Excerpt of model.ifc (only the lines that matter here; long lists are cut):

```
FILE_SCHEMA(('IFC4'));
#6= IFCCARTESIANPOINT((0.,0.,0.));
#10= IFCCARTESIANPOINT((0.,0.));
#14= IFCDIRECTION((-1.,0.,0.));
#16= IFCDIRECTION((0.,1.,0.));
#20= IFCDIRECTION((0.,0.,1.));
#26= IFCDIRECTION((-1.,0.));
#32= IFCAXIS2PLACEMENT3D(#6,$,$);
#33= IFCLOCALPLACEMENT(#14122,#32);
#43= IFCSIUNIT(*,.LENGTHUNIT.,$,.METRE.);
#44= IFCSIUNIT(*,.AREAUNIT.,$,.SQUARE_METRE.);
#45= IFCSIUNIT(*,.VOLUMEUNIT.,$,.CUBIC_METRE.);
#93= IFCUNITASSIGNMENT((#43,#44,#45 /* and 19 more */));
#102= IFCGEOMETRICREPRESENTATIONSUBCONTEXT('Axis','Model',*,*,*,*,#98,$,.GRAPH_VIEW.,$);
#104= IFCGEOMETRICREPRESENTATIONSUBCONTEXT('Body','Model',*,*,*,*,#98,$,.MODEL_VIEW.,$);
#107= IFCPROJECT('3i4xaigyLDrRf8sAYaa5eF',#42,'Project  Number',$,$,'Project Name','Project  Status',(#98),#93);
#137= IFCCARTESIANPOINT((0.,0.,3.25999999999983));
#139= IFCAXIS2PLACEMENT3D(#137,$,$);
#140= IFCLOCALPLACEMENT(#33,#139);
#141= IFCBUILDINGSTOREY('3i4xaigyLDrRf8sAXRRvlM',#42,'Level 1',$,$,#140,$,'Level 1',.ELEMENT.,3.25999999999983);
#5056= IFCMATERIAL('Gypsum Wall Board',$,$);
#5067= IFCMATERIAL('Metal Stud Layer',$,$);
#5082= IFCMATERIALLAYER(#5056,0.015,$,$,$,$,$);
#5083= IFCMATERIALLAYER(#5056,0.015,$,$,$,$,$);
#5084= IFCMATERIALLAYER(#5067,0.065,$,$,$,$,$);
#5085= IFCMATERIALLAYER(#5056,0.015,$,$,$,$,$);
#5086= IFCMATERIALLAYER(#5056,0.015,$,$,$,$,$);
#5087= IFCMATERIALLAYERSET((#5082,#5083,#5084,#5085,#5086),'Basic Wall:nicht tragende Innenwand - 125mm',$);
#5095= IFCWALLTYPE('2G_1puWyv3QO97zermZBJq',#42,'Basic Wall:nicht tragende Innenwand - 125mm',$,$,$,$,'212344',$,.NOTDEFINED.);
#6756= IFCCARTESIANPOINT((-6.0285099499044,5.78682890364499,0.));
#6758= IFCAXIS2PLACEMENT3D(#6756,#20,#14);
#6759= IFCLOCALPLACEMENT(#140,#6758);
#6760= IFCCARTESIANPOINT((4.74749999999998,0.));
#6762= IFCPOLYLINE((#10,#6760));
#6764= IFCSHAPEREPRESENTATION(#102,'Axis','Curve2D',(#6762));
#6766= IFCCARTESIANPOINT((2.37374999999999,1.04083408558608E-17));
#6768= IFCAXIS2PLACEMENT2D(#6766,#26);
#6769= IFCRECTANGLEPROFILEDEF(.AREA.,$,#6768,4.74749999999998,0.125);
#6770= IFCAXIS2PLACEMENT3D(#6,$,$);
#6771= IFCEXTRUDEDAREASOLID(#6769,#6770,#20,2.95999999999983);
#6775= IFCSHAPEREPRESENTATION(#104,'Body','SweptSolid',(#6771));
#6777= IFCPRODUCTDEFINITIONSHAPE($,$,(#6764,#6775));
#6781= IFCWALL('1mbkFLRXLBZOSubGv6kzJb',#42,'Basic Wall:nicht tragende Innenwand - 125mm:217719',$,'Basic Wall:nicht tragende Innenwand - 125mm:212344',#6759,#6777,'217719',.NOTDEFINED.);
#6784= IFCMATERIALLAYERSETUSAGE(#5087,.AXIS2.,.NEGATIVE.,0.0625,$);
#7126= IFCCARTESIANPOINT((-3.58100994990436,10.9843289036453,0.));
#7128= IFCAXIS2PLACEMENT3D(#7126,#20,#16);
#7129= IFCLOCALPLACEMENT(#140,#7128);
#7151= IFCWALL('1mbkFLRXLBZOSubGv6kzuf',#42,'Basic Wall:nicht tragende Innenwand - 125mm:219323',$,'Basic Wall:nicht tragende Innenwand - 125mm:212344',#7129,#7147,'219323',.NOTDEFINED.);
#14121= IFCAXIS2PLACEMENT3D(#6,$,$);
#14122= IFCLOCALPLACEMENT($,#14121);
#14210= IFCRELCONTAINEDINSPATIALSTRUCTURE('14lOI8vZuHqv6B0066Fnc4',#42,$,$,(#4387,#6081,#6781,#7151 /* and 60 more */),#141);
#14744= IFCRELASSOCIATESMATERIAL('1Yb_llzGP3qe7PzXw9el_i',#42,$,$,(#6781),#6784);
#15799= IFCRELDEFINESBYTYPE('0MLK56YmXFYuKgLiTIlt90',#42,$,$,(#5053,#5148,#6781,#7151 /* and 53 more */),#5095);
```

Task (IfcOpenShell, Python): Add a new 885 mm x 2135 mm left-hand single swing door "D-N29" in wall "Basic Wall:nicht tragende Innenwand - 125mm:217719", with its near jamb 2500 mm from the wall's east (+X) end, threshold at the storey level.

```python
import numpy as np
import ifcopenshell
import ifcopenshell.api.feature
import ifcopenshell.api.geometry
import ifcopenshell.api.root
import ifcopenshell.api.spatial
import ifcopenshell.geom
import ifcopenshell.util.element
import ifcopenshell.util.placement
import ifcopenshell.util.representation
import ifcopenshell.util.shape
import ifcopenshell.util.unit

model = ifcopenshell.open("model.ifc")
unit_scale = ifcopenshell.util.unit.calculate_unit_scale(model)
settings = ifcopenshell.geom.settings()


def volume(element):
    """Net volume in cubic metres, openings subtracted."""
    shape = ifcopenshell.geom.create_shape(settings, element)
    return ifcopenshell.util.shape.get_volume(shape.geometry)


wall = model.by_guid("1mbkFLRXLBZOSubGv6kzJb")
storey = ifcopenshell.util.element.get_container(wall, ifc_class="IfcBuildingStorey")
context = ifcopenshell.util.representation.get_context(model, "Model", "Body", "MODEL_VIEW")
before = volume(wall)

width, height, from_end, sill = 0.885, 2.135, 2.5, 0.0  # metres

# The wall runs along its own X axis, and the end named is its -X end.
wall_shape = ifcopenshell.geom.create_shape(settings, wall)
x, y, z = ifcopenshell.util.shape.get_vertices(wall_shape.geometry).T
start = x.min() + from_end
face, thickness = float(y.min()), float(y.max() - y.min())
wall_matrix = ifcopenshell.util.placement.get_local_placement(wall.ObjectPlacement)
level = ifcopenshell.util.placement.get_local_placement(storey.ObjectPlacement)[2, 3]


def in_wall(x, y):
    """Placement at x, y metres in the wall's axes, at sill height."""
    matrix = wall_matrix.copy()
    matrix[:, 3] = wall_matrix @ np.array([x / unit_scale, y / unit_scale, 0.0, 1.0])
    matrix[2, 3] = level + sill / unit_scale
    return matrix


# Opening: a box that overshoots both wall faces by 50 mm.
opening = ifcopenshell.api.root.create_entity(model, ifc_class="IfcOpeningElement", predefined_type="OPENING")
box = ifcopenshell.api.geometry.add_wall_representation(
    model, context=context, length=width, height=height, thickness=thickness + 0.1
)
ifcopenshell.api.geometry.assign_representation(model, product=opening, representation=box)
ifcopenshell.api.geometry.edit_object_placement(model, product=opening, matrix=in_wall(start, face - 0.05), is_si=False)
ifcopenshell.api.feature.add_feature(model, feature=opening, element=wall)

door = ifcopenshell.api.root.create_entity(model, ifc_class="IfcDoor", name="D-N29", predefined_type="DOOR")
door.OverallWidth, door.OverallHeight = width / unit_scale, height / unit_scale
door.OperationType = "SINGLE_SWING_LEFT"
body = ifcopenshell.api.geometry.add_door_representation(
    model,
    context=context,
    overall_width=door.OverallWidth,
    overall_height=door.OverallHeight,
    operation_type="SINGLE_SWING_LEFT",
    lining_properties={"LiningDepth": thickness / unit_scale, "ThresholdDepth": thickness / unit_scale},
)
ifcopenshell.api.geometry.assign_representation(model, product=door, representation=body)
ifcopenshell.api.spatial.assign_container(model, products=[door], relating_structure=storey)
ifcopenshell.api.feature.add_filling(model, opening=opening, element=door)

# The lining spans the wall, so the door starts at the wall face.
ifcopenshell.api.geometry.edit_object_placement(model, product=door, matrix=in_wall(start, face), is_si=False)

after = volume(wall)

print(f"wall volume {before:.3f} -> {after:.3f} m3")

model.write("model_rev.ifc")
```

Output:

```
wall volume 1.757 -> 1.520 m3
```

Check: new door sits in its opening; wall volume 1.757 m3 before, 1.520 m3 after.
